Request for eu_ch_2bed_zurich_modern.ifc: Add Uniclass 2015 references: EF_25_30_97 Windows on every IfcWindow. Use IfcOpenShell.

First a look at what the model holds.

```python
import ifcopenshell

model = ifcopenshell.open("eu_ch_2bed_zurich_modern.ifc")
print(model.schema)
print("classifications:", [c.Name for c in model.by_type("IfcClassification")])
for ifc_class in ("IfcDoor", "IfcRoof", "IfcStair", "IfcWall", "IfcWindow"):
    print(ifc_class, len(model.by_type(ifc_class)))
```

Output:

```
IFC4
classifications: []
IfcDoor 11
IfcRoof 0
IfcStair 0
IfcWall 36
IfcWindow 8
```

```python
import ifcopenshell
import ifcopenshell.api.classification

model = ifcopenshell.open("eu_ch_2bed_zurich_modern.ifc")

system = ifcopenshell.api.classification.add_classification(model, classification="Uniclass 2015")

codes = {
    "IfcWindow": ("EF_25_30_97", "Windows"),
}
for ifc_class, (code, name) in codes.items():
    products = model.by_type(ifc_class)
    ifcopenshell.api.classification.add_reference(
        model, products=products, classification=system, identification=code, name=name
    )
    print(code, len(products))

model.write("eu_ch_2bed_zurich_modern_updated.ifc")
```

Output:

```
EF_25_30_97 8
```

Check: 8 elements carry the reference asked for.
